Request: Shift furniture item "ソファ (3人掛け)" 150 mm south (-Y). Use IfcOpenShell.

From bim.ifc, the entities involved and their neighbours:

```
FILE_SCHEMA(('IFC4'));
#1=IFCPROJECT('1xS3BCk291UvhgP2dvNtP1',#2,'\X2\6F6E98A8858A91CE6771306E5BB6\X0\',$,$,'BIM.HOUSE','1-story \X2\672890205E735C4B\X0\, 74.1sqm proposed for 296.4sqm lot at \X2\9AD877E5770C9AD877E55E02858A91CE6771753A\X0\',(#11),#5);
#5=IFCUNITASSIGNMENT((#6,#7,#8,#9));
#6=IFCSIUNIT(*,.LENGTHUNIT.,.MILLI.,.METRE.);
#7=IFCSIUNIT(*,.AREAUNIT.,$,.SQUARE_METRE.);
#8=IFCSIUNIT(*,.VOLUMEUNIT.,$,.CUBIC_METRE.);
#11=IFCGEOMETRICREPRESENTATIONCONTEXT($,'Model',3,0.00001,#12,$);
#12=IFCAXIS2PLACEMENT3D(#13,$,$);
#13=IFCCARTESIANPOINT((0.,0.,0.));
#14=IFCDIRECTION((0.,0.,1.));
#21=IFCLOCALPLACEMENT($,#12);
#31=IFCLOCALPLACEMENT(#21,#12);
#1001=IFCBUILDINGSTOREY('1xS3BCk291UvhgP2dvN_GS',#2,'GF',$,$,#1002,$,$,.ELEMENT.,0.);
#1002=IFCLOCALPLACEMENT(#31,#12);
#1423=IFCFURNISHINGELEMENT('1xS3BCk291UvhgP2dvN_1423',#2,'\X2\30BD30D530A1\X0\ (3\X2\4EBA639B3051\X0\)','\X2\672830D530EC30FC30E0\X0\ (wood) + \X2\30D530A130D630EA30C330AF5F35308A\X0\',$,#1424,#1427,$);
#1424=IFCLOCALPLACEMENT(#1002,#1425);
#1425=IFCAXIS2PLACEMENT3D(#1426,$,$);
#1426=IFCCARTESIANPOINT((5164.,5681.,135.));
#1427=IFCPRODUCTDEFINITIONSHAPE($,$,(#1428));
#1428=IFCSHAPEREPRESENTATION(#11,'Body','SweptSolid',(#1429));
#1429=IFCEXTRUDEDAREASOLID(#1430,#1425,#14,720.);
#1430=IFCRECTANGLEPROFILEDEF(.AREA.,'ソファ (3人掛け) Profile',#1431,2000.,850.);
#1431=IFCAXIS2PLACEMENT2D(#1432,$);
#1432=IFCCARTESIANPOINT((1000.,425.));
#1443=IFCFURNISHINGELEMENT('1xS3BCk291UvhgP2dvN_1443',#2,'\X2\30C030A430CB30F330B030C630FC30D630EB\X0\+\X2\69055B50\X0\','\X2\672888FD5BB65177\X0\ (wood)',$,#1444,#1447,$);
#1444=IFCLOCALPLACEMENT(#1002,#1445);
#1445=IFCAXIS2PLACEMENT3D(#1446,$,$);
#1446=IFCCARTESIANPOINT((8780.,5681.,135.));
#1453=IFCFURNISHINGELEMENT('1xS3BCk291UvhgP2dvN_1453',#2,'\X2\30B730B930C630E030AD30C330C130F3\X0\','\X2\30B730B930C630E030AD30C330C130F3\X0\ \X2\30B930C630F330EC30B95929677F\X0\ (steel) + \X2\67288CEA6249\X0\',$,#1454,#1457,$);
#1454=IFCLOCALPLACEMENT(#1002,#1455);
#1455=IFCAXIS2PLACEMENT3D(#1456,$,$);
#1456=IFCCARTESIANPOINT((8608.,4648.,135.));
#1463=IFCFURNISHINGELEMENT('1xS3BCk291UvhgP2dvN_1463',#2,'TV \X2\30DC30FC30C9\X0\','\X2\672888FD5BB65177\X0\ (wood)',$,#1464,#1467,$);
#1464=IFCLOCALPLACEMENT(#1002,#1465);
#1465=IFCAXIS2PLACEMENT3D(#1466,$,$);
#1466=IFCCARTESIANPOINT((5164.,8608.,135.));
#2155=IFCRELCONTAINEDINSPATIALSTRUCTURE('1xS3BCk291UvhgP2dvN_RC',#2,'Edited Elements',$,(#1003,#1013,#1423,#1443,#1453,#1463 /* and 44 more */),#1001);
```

```python
import ifcopenshell
import ifcopenshell.api.geometry
import ifcopenshell.util.placement

model = ifcopenshell.open("bim.ifc")

item = model.by_id(1423)
matrix = ifcopenshell.util.placement.get_local_placement(item.ObjectPlacement)
matrix[1, 3] -= 150.0
ifcopenshell.api.geometry.edit_object_placement(model, product=item, matrix=matrix, is_si=False)

print(ifcopenshell.util.placement.get_local_placement(item.ObjectPlacement).round(3) + 0.0)

model.write("bim_v2.ifc")
```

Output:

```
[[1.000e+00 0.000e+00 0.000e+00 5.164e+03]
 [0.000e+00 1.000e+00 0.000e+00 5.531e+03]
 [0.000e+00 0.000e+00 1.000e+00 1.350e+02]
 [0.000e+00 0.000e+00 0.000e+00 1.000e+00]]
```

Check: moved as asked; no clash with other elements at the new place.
